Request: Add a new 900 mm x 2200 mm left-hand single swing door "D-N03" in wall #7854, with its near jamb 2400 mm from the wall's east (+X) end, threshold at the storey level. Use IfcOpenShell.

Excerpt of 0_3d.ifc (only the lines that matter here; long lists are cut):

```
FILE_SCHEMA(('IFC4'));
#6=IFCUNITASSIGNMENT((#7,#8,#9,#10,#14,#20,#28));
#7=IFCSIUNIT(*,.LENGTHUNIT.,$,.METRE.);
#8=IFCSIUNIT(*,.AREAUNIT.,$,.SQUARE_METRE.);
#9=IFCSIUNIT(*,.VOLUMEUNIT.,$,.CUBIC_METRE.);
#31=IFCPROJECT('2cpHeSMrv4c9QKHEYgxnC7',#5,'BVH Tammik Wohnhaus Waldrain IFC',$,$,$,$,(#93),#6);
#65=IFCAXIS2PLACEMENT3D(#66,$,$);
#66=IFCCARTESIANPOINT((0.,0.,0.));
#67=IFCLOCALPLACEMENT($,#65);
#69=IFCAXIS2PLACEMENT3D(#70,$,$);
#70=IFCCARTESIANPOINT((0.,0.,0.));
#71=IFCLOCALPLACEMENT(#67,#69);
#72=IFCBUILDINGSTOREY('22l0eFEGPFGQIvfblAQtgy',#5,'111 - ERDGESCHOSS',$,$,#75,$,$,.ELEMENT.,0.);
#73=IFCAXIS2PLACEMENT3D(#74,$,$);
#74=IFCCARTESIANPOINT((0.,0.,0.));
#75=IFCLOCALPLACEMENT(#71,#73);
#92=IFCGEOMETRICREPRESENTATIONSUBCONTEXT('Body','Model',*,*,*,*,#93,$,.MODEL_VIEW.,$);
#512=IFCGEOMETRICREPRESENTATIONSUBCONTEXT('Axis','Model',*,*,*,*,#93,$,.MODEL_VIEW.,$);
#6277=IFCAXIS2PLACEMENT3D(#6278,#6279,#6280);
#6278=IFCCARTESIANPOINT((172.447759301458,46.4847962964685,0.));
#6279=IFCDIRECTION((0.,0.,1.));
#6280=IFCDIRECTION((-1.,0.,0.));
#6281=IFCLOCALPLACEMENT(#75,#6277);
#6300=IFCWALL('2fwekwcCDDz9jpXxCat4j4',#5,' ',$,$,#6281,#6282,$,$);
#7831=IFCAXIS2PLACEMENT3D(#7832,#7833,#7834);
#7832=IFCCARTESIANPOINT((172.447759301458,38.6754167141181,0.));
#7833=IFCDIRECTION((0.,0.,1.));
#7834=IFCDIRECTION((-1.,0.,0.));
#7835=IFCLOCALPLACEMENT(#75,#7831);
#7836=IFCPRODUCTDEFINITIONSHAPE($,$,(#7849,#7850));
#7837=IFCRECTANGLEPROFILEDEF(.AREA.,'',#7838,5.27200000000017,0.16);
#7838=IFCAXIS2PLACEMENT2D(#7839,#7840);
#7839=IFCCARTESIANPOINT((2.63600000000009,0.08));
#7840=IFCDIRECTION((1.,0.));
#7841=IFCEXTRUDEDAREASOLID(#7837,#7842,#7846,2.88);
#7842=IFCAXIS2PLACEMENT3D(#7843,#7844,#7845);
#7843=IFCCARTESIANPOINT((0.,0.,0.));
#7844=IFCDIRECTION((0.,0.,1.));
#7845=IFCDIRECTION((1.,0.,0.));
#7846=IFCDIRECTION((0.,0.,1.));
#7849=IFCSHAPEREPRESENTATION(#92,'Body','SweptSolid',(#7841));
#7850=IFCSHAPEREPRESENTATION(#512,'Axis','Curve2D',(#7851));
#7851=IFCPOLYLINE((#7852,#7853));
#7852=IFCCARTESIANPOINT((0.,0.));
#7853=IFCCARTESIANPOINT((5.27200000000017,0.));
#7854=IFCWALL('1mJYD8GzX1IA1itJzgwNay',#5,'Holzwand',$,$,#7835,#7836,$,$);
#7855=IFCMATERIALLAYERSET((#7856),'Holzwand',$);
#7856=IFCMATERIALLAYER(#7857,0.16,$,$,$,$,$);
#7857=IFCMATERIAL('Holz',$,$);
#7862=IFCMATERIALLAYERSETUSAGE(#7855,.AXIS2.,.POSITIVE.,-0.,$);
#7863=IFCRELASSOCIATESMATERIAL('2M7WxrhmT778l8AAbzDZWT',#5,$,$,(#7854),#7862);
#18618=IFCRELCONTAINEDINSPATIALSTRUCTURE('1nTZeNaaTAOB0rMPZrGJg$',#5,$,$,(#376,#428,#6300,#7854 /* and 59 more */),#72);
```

```python
import numpy as np
import ifcopenshell
import ifcopenshell.api.feature
import ifcopenshell.api.geometry
import ifcopenshell.api.root
import ifcopenshell.api.spatial
import ifcopenshell.geom
import ifcopenshell.util.element
import ifcopenshell.util.placement
import ifcopenshell.util.representation
import ifcopenshell.util.shape
import ifcopenshell.util.unit

model = ifcopenshell.open("0_3d.ifc")
unit_scale = ifcopenshell.util.unit.calculate_unit_scale(model)
settings = ifcopenshell.geom.settings()


def volume(element):
    """Net volume in cubic metres, openings subtracted."""
    shape = ifcopenshell.geom.create_shape(settings, element)
    return ifcopenshell.util.shape.get_volume(shape.geometry)


wall = model.by_guid("1mJYD8GzX1IA1itJzgwNay")
storey = ifcopenshell.util.element.get_container(wall, ifc_class="IfcBuildingStorey")
context = ifcopenshell.util.representation.get_context(model, "Model", "Body", "MODEL_VIEW")
before = volume(wall)

width, height, from_end, sill = 0.9, 2.2, 2.4, 0.0  # metres

# The wall runs along its own X axis, and the end named is its -X end.
wall_shape = ifcopenshell.geom.create_shape(settings, wall)
x, y, z = ifcopenshell.util.shape.get_vertices(wall_shape.geometry).T
start = x.min() + from_end
face, thickness = float(y.min()), float(y.max() - y.min())
wall_matrix = ifcopenshell.util.placement.get_local_placement(wall.ObjectPlacement)
level = ifcopenshell.util.placement.get_local_placement(storey.ObjectPlacement)[2, 3]


def in_wall(x, y):
    """Placement at x, y metres in the wall's axes, at sill height."""
    matrix = wall_matrix.copy()
    matrix[:, 3] = wall_matrix @ np.array([x / unit_scale, y / unit_scale, 0.0, 1.0])
    matrix[2, 3] = level + sill / unit_scale
    return matrix


# Opening: a box that overshoots both wall faces by 50 mm.
opening = ifcopenshell.api.root.create_entity(model, ifc_class="IfcOpeningElement", predefined_type="OPENING")
box = ifcopenshell.api.geometry.add_wall_representation(
    model, context=context, length=width, height=height, thickness=thickness + 0.1
)
ifcopenshell.api.geometry.assign_representation(model, product=opening, representation=box)
ifcopenshell.api.geometry.edit_object_placement(model, product=opening, matrix=in_wall(start, face - 0.05), is_si=False)
ifcopenshell.api.feature.add_feature(model, feature=opening, element=wall)

door = ifcopenshell.api.root.create_entity(model, ifc_class="IfcDoor", name="D-N03", predefined_type="DOOR")
door.OverallWidth, door.OverallHeight = width / unit_scale, height / unit_scale
door.OperationType = "SINGLE_SWING_LEFT"
body = ifcopenshell.api.geometry.add_door_representation(
    model,
    context=context,
    overall_width=door.OverallWidth,
    overall_height=door.OverallHeight,
    operation_type="SINGLE_SWING_LEFT",
    lining_properties={"LiningDepth": thickness / unit_scale, "ThresholdDepth": thickness / unit_scale},
)
ifcopenshell.api.geometry.assign_representation(model, product=door, representation=body)
ifcopenshell.api.spatial.assign_container(model, products=[door], relating_structure=storey)
ifcopenshell.api.feature.add_filling(model, opening=opening, element=door)

# The lining spans the wall, so the door starts at the wall face.
ifcopenshell.api.geometry.edit_object_placement(model, product=door, matrix=in_wall(start, face), is_si=False)

after = volume(wall)

print(f"wall volume {before:.3f} -> {after:.3f} m3")

model.write("0_3d_edited.ifc")
```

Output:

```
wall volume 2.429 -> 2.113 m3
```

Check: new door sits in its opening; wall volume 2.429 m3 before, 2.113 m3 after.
